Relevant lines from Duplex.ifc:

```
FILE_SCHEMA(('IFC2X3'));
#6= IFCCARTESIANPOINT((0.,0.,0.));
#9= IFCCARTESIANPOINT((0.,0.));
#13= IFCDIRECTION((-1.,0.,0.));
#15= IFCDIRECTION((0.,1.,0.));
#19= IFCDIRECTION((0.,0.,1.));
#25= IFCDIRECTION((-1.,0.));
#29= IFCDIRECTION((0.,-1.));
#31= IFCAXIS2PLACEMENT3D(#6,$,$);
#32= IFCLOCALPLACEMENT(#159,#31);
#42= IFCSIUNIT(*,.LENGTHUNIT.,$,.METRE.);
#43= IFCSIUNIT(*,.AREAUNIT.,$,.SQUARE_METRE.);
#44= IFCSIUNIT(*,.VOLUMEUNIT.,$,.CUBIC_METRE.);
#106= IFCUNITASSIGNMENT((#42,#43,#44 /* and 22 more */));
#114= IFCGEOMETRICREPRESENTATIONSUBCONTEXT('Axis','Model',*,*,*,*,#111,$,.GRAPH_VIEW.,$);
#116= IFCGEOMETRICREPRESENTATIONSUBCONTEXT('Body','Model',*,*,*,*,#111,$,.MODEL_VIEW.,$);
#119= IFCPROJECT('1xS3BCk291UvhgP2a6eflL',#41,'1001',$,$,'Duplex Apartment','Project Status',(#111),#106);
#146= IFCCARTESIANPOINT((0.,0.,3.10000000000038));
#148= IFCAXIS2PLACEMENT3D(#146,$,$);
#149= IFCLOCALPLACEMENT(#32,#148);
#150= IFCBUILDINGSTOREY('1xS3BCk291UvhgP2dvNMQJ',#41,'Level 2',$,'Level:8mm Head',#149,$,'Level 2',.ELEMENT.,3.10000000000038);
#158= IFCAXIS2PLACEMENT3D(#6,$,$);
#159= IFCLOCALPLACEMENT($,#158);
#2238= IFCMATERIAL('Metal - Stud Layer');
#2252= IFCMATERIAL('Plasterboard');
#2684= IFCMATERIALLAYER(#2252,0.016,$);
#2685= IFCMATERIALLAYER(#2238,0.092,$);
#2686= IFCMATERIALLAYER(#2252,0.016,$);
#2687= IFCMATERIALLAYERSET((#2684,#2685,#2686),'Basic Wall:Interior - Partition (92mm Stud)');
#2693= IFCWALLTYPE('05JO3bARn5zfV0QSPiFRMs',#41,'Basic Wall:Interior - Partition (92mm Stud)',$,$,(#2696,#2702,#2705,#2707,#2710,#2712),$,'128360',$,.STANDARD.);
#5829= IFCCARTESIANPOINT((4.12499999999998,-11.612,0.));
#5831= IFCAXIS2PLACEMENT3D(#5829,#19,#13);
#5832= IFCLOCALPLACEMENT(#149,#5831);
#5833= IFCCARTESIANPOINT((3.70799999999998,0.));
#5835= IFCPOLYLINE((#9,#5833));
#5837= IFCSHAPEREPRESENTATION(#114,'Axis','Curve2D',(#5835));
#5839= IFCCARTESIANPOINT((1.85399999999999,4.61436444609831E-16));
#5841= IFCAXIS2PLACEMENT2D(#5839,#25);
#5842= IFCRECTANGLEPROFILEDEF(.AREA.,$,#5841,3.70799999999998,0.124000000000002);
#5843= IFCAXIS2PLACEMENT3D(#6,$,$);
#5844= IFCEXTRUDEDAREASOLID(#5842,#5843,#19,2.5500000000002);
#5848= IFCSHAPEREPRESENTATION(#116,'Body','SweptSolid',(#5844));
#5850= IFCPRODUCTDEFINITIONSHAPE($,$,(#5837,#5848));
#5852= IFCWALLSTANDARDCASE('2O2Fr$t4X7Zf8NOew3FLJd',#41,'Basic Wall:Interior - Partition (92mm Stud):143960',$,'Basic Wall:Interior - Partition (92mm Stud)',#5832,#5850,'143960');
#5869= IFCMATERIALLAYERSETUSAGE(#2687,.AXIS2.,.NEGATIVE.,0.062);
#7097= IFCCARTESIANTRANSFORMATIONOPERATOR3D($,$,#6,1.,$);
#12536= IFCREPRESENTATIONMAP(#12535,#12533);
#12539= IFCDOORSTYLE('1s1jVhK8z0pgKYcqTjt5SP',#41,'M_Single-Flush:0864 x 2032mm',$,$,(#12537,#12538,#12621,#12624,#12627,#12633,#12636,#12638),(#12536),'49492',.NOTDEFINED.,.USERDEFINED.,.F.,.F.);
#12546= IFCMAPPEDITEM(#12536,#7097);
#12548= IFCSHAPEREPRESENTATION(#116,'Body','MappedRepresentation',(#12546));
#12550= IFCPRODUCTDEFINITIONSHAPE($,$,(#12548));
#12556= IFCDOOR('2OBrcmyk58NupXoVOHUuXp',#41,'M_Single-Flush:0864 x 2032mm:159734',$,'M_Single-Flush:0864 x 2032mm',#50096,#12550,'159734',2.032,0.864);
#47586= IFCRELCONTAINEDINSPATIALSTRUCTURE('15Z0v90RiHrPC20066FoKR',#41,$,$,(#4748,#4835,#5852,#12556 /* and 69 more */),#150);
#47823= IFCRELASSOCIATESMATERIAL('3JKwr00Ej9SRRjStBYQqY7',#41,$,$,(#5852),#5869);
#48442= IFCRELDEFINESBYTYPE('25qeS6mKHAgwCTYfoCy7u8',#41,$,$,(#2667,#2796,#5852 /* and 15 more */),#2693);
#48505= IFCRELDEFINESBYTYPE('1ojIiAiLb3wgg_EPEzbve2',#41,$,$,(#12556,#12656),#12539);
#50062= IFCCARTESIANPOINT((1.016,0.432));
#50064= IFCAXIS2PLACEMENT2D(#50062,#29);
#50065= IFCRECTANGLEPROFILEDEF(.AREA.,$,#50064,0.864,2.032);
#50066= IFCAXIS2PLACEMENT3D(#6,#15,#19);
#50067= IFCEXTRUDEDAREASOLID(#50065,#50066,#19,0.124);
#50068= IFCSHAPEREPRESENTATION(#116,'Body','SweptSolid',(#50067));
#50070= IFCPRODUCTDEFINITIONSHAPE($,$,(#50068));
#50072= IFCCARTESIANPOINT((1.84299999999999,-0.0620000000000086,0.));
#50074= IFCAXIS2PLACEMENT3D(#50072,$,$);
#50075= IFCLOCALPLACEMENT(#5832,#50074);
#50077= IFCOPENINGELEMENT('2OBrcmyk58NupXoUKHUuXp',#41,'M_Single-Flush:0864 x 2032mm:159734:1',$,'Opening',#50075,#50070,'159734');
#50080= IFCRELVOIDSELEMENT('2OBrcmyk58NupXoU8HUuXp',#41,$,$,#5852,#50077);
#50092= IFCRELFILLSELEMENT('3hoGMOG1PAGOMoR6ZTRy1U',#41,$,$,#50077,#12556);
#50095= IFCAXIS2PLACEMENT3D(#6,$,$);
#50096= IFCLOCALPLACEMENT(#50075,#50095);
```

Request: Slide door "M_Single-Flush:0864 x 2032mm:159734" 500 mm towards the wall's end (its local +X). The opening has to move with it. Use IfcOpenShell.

```python
import ifcopenshell
import ifcopenshell.api.geometry
import ifcopenshell.util.placement

model = ifcopenshell.open("Duplex.ifc")

door = model.by_guid("2OBrcmyk58NupXoVOHUuXp")
opening = door.FillsVoids[0].RelatingOpeningElement
wall = opening.VoidsElements[0].RelatingBuildingElement

wall_matrix = ifcopenshell.util.placement.get_local_placement(wall.ObjectPlacement)
shift = wall_matrix[:3, 0] * 0.5
before = ifcopenshell.util.placement.get_local_placement(door.ObjectPlacement)[:3, 3].copy()

# The door is placed relative to its opening, so it follows when the opening moves.
matrix = ifcopenshell.util.placement.get_local_placement(opening.ObjectPlacement)
matrix[:3, 3] += shift
ifcopenshell.api.geometry.edit_object_placement(
    model, product=opening, matrix=matrix, is_si=False, should_transform_children=True
)

after = ifcopenshell.util.placement.get_local_placement(door.ObjectPlacement)[:3, 3]
print("door moved by", (after - before).round(3) + 0.0)

model.write("Duplex-out.ifc")
```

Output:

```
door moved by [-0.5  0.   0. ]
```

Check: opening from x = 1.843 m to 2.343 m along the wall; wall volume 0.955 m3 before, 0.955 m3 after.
